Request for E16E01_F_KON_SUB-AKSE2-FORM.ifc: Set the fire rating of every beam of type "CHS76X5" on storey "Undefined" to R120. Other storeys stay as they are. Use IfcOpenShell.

First a look at what the model holds.

```python
import ifcopenshell
import ifcopenshell.util.element

model = ifcopenshell.open("E16E01_F_KON_SUB-AKSE2-FORM.ifc")
print(model.schema)
storey = next(s for s in model.by_type("IfcBuildingStorey") if s.Name == "Undefined")
beams = [e for e in ifcopenshell.util.element.get_decomposition(storey) if e.is_a("IfcBeam")]
seen = {}
for e in beams:
    element_type = ifcopenshell.util.element.get_type(e)
    key = (element_type.Name if element_type != e and element_type else None, ifcopenshell.util.element.get_pset(e, "Pset_BeamCommon", "FireRating"))
    seen[key] = seen.get(key, 0) + 1
for (name, value), count in sorted(seen.items(), key=str):
    print(count, "x", name, "|", value)
```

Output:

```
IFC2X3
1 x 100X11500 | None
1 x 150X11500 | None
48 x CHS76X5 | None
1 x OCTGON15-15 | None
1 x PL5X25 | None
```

```python
import ifcopenshell
import ifcopenshell.api.pset
import ifcopenshell.util.element

model = ifcopenshell.open("E16E01_F_KON_SUB-AKSE2-FORM.ifc")

storey = next(s for s in model.by_type("IfcBuildingStorey") if s.Name == "Undefined")
beams = [e for e in ifcopenshell.util.element.get_decomposition(storey) if e.is_a("IfcBeam")]

count = 0
for e in beams:
    element_type = ifcopenshell.util.element.get_type(e)
    if element_type in (None, e) or element_type.Name != "CHS76X5":
        continue
    found = ifcopenshell.util.element.get_pset(e, "Pset_BeamCommon", should_inherit=False)
    if found:
        pset = model.by_id(found["id"])
        if len(ifcopenshell.util.element.get_elements_by_pset(pset)) > 1:
            pset = ifcopenshell.api.pset.unshare_pset(model, products=[e], pset=pset)[0]
    else:
        pset = ifcopenshell.api.pset.add_pset(model, product=e, name="Pset_BeamCommon")
    ifcopenshell.api.pset.edit_pset(model, pset=pset, properties={"FireRating": "R120"})
    count += 1

print(count, "beams updated")

model.write("E16E01_F_KON_SUB-AKSE2-FORM_edited.ifc")
```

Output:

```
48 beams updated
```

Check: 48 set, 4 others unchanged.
